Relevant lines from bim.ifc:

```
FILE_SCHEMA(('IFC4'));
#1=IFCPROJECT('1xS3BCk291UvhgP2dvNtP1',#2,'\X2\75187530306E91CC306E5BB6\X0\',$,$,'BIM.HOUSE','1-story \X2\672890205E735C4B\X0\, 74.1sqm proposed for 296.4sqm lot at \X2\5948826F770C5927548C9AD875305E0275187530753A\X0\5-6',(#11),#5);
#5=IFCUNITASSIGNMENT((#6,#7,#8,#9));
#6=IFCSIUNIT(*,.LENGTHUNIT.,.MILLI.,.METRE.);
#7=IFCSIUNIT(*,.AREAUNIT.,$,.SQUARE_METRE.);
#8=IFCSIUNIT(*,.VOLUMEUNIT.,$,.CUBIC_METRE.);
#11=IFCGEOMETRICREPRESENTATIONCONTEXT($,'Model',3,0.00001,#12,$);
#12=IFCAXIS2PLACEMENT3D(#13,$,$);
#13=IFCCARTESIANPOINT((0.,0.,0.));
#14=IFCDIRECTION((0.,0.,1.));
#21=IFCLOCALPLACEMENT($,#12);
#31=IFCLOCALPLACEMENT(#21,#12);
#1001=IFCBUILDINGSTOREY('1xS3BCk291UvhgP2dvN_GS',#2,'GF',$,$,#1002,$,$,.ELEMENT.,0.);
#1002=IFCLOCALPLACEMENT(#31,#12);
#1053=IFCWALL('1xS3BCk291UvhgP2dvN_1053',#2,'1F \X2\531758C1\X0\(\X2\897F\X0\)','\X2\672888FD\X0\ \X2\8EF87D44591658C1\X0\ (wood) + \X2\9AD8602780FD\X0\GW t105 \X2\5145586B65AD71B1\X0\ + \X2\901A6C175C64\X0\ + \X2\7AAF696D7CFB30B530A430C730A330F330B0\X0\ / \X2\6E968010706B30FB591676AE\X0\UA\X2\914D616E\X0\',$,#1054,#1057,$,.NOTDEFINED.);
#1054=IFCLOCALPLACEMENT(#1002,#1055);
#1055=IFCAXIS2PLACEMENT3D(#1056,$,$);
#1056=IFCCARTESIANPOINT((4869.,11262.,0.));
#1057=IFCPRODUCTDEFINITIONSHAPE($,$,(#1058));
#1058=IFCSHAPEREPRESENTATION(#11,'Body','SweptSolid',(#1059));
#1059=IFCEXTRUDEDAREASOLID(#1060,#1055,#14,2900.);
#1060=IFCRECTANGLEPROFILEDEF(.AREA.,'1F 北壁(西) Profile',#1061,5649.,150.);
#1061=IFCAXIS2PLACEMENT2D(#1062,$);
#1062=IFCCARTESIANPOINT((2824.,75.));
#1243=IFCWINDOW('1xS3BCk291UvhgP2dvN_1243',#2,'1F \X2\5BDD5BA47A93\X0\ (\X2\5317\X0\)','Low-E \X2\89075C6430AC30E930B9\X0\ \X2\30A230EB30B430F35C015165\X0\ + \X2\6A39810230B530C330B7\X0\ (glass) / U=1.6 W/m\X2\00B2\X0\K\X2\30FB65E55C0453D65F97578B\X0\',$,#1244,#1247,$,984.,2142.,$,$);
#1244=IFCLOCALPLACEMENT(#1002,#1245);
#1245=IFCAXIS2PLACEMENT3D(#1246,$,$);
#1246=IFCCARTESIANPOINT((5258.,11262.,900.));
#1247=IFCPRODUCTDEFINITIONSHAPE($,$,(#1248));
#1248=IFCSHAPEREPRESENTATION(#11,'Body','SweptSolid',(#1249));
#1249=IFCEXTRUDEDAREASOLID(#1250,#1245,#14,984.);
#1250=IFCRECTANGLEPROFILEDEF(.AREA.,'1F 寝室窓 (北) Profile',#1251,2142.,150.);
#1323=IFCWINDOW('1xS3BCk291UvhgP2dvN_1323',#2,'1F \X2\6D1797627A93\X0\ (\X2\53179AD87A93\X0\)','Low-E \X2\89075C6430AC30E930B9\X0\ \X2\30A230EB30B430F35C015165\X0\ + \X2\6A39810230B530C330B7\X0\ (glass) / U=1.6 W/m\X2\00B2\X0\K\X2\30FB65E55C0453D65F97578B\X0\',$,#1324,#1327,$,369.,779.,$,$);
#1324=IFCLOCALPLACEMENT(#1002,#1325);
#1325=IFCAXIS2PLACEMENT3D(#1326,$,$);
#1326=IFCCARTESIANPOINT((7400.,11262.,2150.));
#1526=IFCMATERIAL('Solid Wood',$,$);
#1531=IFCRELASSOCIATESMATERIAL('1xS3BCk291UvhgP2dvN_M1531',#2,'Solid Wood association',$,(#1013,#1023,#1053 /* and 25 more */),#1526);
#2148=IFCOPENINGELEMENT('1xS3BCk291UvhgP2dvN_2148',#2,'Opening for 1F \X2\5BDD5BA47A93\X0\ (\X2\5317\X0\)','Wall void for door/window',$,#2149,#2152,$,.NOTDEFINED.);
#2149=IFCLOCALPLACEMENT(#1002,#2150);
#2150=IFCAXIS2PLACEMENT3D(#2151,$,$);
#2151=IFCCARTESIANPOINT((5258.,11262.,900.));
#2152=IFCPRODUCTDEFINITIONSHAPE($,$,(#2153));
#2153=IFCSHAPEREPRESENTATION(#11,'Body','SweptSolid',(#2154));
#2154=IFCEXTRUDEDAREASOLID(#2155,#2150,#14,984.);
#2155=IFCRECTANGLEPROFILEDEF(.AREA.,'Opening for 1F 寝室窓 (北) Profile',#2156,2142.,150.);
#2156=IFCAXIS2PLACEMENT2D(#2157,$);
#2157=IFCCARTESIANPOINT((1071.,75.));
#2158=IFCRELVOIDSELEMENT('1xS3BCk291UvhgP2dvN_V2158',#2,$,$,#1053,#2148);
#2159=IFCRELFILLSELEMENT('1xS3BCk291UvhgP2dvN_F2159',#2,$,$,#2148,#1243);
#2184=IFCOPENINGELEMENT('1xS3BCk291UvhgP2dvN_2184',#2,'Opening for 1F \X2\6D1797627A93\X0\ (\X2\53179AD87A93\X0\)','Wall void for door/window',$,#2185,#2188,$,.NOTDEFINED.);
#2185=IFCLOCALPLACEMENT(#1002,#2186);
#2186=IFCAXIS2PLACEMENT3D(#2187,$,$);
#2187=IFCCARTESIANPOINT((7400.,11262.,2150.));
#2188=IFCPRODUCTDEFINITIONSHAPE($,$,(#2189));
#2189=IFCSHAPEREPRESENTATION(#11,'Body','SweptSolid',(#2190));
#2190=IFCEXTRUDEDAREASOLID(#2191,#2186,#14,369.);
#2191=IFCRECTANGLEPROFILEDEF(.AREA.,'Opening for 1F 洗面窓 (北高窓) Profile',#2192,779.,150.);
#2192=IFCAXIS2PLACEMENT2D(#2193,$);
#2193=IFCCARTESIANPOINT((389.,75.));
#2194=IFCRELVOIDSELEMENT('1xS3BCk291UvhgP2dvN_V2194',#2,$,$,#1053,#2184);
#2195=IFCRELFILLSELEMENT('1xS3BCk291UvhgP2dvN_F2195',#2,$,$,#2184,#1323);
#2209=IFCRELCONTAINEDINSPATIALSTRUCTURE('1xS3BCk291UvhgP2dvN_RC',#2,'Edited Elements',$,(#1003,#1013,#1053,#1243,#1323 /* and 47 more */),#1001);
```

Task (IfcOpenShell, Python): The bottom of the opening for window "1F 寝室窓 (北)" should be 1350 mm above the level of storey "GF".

```python
import numpy as np
import ifcopenshell
import ifcopenshell.api.geometry
import ifcopenshell.geom
import ifcopenshell.util.element
import ifcopenshell.util.placement
import ifcopenshell.util.shape
import ifcopenshell.util.unit

model = ifcopenshell.open("bim.ifc")
unit_scale = ifcopenshell.util.unit.calculate_unit_scale(model)

window = model.by_id(1243)
opening = window.FillsVoids[0].RelatingOpeningElement
storey = ifcopenshell.util.element.get_container(window, ifc_class="IfcBuildingStorey")
level = ifcopenshell.util.placement.get_local_placement(storey.ObjectPlacement)[2, 3]

# The opening's origin need not be at the sill, so measure its lowest point.
shape = ifcopenshell.geom.create_shape(ifcopenshell.geom.settings(), opening)
bottom = ifcopenshell.util.shape.get_shape_bottom_elevation(shape, shape.geometry) / unit_scale
dz = level + 1.35 / unit_scale - bottom

shift = np.array([0.0, 0.0, dz])
# The window is not placed relative to its opening, so move both.
for product in (opening, window):
    matrix = ifcopenshell.util.placement.get_local_placement(product.ObjectPlacement)
    matrix[:3, 3] += shift
    ifcopenshell.api.geometry.edit_object_placement(model, product=product, matrix=matrix, is_si=False)

print(f"moved by {dz * unit_scale:+.3f} m")

model.write("bim_rev.ifc")
```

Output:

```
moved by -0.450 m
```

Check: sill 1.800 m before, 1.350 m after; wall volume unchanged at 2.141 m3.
